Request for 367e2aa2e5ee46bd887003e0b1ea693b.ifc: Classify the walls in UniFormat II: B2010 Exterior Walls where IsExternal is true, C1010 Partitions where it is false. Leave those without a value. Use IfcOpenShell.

First a look at what the model holds.

```python
import ifcopenshell
import ifcopenshell.util.element

model = ifcopenshell.open("367e2aa2e5ee46bd887003e0b1ea693b.ifc")
print(model.schema)
print("classifications:", [c.Name for c in model.by_type("IfcClassification")])
values = [ifcopenshell.util.element.get_pset(e, "Pset_WallCommon", "IsExternal") for e in model.by_type("IfcWall")]
for value in (True, False, None):
    print("IsExternal", value, values.count(value))
```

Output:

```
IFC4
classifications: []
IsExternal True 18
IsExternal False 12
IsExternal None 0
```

```python
import ifcopenshell
import ifcopenshell.api.classification
import ifcopenshell.util.element

model = ifcopenshell.open("367e2aa2e5ee46bd887003e0b1ea693b.ifc")

system = ifcopenshell.api.classification.add_classification(model, classification="UniFormat II")

walls = model.by_type("IfcWall")
external = {e: ifcopenshell.util.element.get_pset(e, "Pset_WallCommon", "IsExternal") for e in walls}
for flag, code, name in ((True, "B2010", "Exterior Walls"), (False, "C1010", "Partitions")):
    products = [e for e in walls if external[e] is flag]
    ifcopenshell.api.classification.add_reference(
        model, products=products, classification=system, identification=code, name=name
    )
    print(code, len(products))

model.write("367e2aa2e5ee46bd887003e0b1ea693b_edited.ifc")
```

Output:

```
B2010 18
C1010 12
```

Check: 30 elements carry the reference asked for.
